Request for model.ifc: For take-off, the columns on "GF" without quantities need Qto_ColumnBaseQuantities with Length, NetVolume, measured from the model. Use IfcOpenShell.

First a look at what the model holds.

```python
import ifcopenshell
import ifcopenshell.util.element
import ifcopenshell.util.unit

model = ifcopenshell.open("model.ifc")
print(model.schema)
for unit_type in ("LENGTHUNIT", "AREAUNIT", "VOLUMEUNIT"):
    print(unit_type, ifcopenshell.util.unit.calculate_unit_scale(model, unit_type))
storey = next(s for s in model.by_type("IfcBuildingStorey") if s.Name == "GF")
columns = [e for e in ifcopenshell.util.element.get_decomposition(storey) if e.is_a("IfcColumn")]
for e in sorted(columns, key=lambda e: e.id()):
    print(e.id(), e.is_a(), e.Name, list(ifcopenshell.util.element.get_psets(e, qtos_only=True)), sep=" | ")
```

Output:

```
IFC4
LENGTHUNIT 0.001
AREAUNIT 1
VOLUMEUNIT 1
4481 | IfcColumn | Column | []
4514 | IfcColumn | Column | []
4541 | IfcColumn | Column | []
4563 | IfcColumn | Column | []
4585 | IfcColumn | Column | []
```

```python
import ifcopenshell
import ifcopenshell.api.pset
import ifcopenshell.geom
import ifcopenshell.util.element
import ifcopenshell.util.shape
import ifcopenshell.util.unit

model = ifcopenshell.open("model.ifc")
unit_scale = ifcopenshell.util.unit.calculate_unit_scale(model)
volume_scale = ifcopenshell.util.unit.calculate_unit_scale(model, "VOLUMEUNIT")
settings = ifcopenshell.geom.settings()

storey = next(s for s in model.by_type("IfcBuildingStorey") if s.Name == "GF")
columns = [e for e in ifcopenshell.util.element.get_decomposition(storey) if e.is_a("IfcColumn")]

for e in sorted(columns, key=lambda e: e.id()):
    if ifcopenshell.util.element.get_psets(e, qtos_only=True, should_inherit=False):
        continue
    # Geometry comes back in metres, in the element's own axes.
    shape = ifcopenshell.geom.create_shape(settings, e)
    values = {
        "Length": ifcopenshell.util.shape.get_z(shape.geometry) / unit_scale,
        "NetVolume": ifcopenshell.util.shape.get_volume(shape.geometry) / volume_scale,
    }
    qto = ifcopenshell.api.pset.add_qto(model, product=e, name="Qto_ColumnBaseQuantities")
    ifcopenshell.api.pset.edit_qto(model, qto=qto, properties=values)
    print(e.id(), {k: round(v, 3) for k, v in values.items()})

model.write("model-out.ifc")
```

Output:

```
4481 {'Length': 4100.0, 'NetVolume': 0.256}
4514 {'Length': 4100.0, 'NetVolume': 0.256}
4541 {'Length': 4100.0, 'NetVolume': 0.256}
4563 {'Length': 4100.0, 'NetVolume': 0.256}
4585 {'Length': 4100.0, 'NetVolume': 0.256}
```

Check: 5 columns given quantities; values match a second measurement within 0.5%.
